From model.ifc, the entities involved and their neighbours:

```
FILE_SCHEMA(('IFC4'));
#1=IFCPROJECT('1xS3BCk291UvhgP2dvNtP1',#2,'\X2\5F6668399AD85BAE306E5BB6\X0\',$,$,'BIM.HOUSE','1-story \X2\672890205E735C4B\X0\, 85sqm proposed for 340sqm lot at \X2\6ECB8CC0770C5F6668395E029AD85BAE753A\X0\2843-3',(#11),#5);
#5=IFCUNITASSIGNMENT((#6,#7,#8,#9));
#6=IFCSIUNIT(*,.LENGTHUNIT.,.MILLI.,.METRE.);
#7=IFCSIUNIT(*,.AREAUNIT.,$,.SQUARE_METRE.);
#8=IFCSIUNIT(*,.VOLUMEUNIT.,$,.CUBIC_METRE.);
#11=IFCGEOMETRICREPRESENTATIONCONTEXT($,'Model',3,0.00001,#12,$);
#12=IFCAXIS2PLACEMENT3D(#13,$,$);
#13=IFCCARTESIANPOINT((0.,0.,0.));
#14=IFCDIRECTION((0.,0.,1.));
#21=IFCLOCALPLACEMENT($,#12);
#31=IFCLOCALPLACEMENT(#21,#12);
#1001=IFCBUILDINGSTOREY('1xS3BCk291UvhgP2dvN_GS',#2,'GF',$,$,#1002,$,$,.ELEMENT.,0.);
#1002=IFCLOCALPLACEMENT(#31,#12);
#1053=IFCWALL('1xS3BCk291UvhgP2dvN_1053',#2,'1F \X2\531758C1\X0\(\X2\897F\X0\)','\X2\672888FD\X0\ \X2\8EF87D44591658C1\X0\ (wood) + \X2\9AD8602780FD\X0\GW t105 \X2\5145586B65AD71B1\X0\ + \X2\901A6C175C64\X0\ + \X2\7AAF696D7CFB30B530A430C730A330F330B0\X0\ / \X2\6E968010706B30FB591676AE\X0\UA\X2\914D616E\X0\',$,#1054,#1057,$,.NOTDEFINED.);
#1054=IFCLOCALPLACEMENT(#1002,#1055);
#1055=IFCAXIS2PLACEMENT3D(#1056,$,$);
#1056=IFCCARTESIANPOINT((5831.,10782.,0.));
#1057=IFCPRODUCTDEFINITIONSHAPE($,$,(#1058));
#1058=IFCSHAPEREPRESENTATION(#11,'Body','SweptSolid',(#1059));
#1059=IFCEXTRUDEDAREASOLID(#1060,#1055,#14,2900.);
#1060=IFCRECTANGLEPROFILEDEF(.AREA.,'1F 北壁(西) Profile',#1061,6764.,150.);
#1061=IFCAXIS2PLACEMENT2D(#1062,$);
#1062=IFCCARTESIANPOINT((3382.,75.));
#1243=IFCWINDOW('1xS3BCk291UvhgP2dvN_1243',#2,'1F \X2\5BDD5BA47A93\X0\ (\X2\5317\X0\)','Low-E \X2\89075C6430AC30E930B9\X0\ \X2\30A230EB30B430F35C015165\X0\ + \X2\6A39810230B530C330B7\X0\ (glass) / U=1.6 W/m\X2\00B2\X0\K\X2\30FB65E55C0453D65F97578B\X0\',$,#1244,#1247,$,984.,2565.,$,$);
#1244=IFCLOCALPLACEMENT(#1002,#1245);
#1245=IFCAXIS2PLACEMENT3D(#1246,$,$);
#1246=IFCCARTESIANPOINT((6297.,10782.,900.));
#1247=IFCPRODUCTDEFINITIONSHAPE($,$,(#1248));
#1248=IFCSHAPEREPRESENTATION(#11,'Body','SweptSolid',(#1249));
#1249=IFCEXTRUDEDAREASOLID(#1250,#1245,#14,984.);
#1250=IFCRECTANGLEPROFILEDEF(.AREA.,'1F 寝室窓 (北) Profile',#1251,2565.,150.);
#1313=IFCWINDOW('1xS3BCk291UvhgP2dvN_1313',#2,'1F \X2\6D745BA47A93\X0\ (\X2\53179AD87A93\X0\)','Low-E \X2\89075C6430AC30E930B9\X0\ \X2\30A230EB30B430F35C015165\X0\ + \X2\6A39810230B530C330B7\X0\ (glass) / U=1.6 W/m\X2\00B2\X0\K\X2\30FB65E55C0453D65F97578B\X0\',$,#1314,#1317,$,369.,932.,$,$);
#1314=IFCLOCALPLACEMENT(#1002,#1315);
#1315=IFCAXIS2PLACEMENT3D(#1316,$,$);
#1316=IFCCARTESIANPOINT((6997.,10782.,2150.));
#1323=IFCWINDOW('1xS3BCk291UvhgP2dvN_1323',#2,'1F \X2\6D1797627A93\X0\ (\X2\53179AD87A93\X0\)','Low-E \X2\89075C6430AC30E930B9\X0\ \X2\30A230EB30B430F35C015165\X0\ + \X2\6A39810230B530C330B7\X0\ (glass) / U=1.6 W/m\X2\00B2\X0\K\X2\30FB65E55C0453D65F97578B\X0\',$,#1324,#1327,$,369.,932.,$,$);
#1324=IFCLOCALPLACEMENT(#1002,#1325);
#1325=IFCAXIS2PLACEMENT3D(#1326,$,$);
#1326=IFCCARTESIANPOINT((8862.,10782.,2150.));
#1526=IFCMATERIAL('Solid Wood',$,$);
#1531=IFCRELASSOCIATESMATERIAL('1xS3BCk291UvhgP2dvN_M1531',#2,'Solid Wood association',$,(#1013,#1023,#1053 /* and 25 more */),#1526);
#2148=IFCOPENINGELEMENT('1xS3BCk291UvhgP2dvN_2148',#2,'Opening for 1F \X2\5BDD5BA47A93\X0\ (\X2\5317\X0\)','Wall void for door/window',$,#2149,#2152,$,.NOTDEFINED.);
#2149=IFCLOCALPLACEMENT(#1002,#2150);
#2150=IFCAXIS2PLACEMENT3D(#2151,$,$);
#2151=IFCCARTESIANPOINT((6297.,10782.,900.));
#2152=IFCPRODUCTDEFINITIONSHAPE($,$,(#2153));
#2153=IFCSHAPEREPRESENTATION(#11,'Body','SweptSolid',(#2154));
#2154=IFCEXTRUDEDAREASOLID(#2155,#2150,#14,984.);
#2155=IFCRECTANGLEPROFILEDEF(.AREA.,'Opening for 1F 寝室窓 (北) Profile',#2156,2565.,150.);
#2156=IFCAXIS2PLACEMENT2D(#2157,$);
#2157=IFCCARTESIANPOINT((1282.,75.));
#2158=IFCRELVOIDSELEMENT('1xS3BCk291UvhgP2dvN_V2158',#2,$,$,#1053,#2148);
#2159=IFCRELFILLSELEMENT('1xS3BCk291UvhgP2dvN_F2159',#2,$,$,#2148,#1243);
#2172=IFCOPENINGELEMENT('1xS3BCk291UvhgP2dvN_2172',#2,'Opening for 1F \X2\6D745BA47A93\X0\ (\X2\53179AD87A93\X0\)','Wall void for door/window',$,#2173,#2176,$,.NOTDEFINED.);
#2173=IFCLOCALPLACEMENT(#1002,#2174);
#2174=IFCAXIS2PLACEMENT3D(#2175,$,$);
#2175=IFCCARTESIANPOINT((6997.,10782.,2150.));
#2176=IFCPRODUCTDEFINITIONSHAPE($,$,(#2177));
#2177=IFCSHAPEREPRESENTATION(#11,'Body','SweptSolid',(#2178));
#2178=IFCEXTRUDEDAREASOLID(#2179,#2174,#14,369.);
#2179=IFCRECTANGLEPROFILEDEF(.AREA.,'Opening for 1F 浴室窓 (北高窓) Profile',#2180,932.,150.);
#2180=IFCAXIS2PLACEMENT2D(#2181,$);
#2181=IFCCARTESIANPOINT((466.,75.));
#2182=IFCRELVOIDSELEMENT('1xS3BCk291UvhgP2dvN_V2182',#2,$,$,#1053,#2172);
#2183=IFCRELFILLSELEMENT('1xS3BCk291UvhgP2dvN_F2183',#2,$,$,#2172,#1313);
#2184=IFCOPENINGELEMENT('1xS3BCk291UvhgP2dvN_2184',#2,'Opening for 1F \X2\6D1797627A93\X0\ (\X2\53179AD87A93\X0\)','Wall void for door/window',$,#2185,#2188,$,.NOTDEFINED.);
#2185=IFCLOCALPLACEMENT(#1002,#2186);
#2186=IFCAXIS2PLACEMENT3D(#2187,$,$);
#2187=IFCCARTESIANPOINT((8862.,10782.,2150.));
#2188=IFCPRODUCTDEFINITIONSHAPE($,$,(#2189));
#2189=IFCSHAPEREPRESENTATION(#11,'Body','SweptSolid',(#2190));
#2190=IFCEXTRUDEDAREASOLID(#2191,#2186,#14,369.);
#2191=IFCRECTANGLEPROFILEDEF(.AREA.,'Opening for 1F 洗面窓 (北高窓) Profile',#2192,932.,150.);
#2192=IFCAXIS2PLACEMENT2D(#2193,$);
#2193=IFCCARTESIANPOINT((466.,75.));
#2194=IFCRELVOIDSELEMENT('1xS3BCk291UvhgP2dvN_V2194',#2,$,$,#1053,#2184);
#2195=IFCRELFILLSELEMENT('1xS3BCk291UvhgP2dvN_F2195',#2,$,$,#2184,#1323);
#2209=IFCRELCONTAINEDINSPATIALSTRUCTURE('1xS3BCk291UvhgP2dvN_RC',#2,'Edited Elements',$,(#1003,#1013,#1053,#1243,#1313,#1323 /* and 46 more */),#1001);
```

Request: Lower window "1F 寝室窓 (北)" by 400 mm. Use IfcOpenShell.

```python
import numpy as np
import ifcopenshell
import ifcopenshell.api.geometry
import ifcopenshell.util.placement
import ifcopenshell.util.unit

model = ifcopenshell.open("model.ifc")
unit_scale = ifcopenshell.util.unit.calculate_unit_scale(model)

window = model.by_guid("1xS3BCk291UvhgP2dvN_1243")
opening = window.FillsVoids[0].RelatingOpeningElement
dz = -400.0

shift = np.array([0.0, 0.0, dz])
# The window is not placed relative to its opening, so move both.
for product in (opening, window):
    matrix = ifcopenshell.util.placement.get_local_placement(product.ObjectPlacement)
    matrix[:3, 3] += shift
    ifcopenshell.api.geometry.edit_object_placement(model, product=product, matrix=matrix, is_si=False)

print(f"moved by {dz * unit_scale:+.3f} m")

model.write("model_edited.ifc")
```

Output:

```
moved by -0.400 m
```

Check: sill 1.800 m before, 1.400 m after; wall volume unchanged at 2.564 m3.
